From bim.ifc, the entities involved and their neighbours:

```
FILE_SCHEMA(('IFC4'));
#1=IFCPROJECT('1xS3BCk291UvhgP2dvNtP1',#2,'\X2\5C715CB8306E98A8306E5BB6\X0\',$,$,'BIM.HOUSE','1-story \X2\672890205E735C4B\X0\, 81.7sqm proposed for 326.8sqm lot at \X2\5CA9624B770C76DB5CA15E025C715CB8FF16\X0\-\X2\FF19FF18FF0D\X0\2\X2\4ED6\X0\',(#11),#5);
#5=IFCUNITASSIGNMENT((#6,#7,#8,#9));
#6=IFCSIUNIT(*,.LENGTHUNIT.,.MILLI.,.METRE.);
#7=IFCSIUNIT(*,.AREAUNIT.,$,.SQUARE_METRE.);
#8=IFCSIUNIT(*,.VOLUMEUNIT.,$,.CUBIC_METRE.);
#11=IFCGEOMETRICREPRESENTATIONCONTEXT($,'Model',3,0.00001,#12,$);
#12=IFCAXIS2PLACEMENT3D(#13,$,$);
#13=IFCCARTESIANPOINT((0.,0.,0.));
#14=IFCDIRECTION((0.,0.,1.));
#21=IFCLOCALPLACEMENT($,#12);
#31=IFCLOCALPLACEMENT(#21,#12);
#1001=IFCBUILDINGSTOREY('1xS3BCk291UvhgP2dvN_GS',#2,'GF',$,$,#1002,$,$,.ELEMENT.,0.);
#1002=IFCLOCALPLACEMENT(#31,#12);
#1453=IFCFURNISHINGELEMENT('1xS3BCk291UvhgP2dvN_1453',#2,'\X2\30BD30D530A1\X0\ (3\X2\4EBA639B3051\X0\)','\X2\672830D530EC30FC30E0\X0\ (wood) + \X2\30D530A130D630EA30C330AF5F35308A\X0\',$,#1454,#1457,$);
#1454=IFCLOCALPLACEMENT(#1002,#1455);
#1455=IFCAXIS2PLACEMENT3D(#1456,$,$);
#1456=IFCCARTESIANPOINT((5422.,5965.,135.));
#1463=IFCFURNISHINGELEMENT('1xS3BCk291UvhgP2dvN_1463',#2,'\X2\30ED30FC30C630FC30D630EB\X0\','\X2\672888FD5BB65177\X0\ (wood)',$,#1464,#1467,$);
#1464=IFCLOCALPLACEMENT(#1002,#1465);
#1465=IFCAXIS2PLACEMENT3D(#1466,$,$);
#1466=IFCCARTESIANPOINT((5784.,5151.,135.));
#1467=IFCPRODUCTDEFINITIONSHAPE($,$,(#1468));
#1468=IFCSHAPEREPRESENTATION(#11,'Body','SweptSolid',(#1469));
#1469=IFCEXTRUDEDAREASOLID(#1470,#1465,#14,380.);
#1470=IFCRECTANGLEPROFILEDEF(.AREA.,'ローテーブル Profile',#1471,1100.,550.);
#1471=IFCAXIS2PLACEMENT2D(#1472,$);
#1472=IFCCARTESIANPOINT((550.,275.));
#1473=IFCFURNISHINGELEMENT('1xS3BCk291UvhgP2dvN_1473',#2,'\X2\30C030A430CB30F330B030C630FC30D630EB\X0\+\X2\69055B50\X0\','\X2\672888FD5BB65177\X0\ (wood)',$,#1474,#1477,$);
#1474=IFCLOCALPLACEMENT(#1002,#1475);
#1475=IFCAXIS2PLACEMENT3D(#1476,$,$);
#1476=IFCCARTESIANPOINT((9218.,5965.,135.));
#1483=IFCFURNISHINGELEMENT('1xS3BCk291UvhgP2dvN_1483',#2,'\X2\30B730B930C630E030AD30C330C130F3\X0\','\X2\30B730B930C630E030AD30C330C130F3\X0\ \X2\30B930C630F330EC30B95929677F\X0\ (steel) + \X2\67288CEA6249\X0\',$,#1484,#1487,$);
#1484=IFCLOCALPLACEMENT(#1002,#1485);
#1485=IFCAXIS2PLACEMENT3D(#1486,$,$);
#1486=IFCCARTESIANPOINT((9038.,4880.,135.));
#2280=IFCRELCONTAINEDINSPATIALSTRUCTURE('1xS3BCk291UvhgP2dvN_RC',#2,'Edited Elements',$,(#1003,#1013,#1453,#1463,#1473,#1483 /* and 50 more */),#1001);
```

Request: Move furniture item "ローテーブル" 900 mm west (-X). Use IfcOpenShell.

```python
import ifcopenshell
import ifcopenshell.api.geometry
import ifcopenshell.util.placement
import ifcopenshell.util.unit

model = ifcopenshell.open("bim.ifc")
unit_scale = ifcopenshell.util.unit.calculate_unit_scale(model)

item = model.by_guid("1xS3BCk291UvhgP2dvN_1463")
matrix = ifcopenshell.util.placement.get_local_placement(item.ObjectPlacement)
matrix[0, 3] -= 0.9 / unit_scale
ifcopenshell.api.geometry.edit_object_placement(model, product=item, matrix=matrix, is_si=False)

print(ifcopenshell.util.placement.get_local_placement(item.ObjectPlacement).round(3) + 0.0)

model.write("bim_edited.ifc")
```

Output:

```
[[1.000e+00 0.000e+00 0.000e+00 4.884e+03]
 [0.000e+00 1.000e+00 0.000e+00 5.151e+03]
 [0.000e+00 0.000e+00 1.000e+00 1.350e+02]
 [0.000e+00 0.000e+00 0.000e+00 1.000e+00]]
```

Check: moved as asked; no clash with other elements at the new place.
